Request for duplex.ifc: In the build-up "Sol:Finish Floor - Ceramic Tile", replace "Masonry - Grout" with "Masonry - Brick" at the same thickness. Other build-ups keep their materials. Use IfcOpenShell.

First a look at what the model holds.

```python
import ifcopenshell
import ifcopenshell.util.element

model = ifcopenshell.open("duplex.ifc")
print(model.schema)
for layer_set in model.by_type("IfcMaterialLayerSet"):
    if layer_set.LayerSetName == "Sol:Finish Floor - Ceramic Tile":
        for layer in layer_set.MaterialLayers:
            print(layer.id(), layer.Material and layer.Material.Name, layer.LayerThickness, sep=" | ")
        print(len(ifcopenshell.util.element.get_elements_by_material(model, layer_set)), "elements and types use it")
print(sorted(m.Name for m in model.by_type("IfcMaterial") if m.Name)[:60])
```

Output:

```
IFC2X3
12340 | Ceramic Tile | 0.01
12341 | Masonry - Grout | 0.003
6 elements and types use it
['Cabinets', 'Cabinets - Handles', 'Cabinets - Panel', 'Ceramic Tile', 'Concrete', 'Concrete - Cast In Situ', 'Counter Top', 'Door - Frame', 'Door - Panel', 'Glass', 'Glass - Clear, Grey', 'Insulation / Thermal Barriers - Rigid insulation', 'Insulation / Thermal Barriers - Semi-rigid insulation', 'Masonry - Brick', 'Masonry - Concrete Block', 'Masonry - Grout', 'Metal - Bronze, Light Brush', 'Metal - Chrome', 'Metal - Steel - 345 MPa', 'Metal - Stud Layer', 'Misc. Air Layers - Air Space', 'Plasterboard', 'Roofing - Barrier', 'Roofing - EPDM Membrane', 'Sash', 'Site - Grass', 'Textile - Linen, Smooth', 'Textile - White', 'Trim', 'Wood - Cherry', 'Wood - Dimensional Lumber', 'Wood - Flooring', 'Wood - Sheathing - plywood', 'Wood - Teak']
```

```python
import ifcopenshell
import ifcopenshell.api.material

model = ifcopenshell.open("duplex.ifc")

layer_set = next(s for s in model.by_type("IfcMaterialLayerSet") if s.LayerSetName == "Sol:Finish Floor - Ceramic Tile")
layer = next(l for l in layer_set.MaterialLayers if l.Material and l.Material.Name == "Masonry - Grout")
material = next(m for m in model.by_type("IfcMaterial") if m.Name == "Masonry - Brick")

# Point this one layer at the other material; renaming the old one would change it everywhere.
ifcopenshell.api.material.edit_layer(model, layer=layer, attributes={}, material=material)

print([l.Material.Name if l.Material else None for l in layer_set.MaterialLayers])

model.write("duplex_updated.ifc")
```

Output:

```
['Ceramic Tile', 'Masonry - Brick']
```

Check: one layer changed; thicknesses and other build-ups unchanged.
